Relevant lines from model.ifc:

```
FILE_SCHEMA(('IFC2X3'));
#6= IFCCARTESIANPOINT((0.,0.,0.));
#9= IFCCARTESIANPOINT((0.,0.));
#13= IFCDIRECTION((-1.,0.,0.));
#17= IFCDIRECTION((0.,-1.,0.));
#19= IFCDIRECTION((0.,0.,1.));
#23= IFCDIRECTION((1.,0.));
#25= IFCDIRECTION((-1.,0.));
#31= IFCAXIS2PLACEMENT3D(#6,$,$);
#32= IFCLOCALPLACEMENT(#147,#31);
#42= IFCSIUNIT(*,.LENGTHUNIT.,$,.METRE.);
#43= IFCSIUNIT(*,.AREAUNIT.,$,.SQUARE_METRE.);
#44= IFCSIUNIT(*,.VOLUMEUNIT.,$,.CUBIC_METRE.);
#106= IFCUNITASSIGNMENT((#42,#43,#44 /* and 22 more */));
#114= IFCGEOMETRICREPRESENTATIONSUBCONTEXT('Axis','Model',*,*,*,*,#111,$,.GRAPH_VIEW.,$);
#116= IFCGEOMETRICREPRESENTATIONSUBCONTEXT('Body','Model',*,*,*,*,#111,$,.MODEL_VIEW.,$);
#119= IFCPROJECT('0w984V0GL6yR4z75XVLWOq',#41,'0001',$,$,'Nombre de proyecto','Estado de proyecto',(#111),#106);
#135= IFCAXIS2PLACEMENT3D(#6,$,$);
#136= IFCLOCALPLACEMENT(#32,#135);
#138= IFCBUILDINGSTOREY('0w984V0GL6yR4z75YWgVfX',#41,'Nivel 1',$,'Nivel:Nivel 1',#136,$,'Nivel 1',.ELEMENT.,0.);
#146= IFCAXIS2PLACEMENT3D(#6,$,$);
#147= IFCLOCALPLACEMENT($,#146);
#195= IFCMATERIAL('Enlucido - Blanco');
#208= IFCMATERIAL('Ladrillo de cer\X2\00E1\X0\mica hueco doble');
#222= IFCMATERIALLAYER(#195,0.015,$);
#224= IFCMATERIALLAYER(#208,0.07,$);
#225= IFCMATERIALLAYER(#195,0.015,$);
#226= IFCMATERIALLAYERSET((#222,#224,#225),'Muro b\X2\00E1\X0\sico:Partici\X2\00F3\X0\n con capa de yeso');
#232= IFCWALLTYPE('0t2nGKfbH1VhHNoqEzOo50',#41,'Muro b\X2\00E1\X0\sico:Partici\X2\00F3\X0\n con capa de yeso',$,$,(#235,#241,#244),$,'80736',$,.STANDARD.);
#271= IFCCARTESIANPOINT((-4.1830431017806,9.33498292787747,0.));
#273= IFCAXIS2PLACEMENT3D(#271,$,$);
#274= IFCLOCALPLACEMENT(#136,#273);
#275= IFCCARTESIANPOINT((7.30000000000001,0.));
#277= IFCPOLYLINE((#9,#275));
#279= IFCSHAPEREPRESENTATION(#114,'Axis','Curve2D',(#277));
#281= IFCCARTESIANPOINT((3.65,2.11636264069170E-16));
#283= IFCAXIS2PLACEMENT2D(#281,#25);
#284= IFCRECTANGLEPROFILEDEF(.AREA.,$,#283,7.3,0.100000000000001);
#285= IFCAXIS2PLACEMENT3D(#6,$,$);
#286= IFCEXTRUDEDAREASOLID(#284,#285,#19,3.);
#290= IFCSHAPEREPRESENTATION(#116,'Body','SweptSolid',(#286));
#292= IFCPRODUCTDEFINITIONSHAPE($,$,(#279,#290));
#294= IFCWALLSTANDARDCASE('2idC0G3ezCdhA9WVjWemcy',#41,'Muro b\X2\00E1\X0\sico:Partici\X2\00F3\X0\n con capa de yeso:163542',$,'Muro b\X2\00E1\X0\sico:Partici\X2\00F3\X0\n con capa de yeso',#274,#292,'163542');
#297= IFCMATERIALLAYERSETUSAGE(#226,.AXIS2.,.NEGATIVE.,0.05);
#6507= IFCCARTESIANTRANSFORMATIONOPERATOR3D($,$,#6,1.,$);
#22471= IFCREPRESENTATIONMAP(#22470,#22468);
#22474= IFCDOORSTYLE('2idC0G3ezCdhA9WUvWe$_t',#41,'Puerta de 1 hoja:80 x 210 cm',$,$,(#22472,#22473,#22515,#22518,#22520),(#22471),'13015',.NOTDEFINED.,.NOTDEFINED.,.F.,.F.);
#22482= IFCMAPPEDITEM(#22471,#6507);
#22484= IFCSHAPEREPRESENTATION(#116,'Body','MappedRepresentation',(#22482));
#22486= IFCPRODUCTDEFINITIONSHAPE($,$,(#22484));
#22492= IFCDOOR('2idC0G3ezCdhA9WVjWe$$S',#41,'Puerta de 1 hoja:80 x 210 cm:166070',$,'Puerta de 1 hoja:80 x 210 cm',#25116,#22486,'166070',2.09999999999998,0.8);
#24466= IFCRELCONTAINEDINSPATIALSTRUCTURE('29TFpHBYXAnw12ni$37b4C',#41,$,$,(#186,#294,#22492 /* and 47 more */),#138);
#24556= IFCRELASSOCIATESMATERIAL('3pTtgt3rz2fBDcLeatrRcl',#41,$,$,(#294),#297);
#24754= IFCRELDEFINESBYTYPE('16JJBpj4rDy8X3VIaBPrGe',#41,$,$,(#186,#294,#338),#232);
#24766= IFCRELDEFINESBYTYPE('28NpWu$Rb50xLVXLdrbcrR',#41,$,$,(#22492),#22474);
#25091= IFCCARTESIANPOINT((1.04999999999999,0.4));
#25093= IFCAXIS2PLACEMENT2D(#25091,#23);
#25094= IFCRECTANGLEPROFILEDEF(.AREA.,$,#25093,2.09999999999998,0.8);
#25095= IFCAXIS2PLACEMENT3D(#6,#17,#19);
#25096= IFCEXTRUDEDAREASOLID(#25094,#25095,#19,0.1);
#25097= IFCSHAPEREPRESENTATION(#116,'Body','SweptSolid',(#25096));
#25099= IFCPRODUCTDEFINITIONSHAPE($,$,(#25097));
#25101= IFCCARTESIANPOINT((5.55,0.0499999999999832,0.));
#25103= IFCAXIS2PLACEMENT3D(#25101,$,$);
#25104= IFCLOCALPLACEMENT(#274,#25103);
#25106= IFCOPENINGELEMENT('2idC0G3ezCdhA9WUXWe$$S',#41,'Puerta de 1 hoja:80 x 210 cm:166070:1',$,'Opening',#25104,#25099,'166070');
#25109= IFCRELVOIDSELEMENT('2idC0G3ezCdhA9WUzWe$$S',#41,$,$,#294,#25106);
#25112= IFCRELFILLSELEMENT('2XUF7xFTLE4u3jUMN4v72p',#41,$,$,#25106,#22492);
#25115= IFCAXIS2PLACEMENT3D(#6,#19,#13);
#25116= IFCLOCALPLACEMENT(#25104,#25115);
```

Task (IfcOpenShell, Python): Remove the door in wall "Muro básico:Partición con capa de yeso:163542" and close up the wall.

```python
import ifcopenshell
import ifcopenshell.api.feature
import ifcopenshell.api.root
import ifcopenshell.geom
import ifcopenshell.util.shape

model = ifcopenshell.open("model.ifc")
settings = ifcopenshell.geom.settings()


def volume(element):
    """Net volume in cubic metres, openings subtracted."""
    shape = ifcopenshell.geom.create_shape(settings, element)
    return ifcopenshell.util.shape.get_volume(shape.geometry)


door = model.by_guid("2idC0G3ezCdhA9WVjWe$$S")
opening = door.FillsVoids[0].RelatingOpeningElement
wall = opening.VoidsElements[0].RelatingBuildingElement
before = volume(wall)

ifcopenshell.api.root.remove_product(model, product=door)
ifcopenshell.api.feature.remove_feature(model, feature=opening)

after = volume(wall)

print(f"wall volume {before:.3f} -> {after:.3f} m3")

model.write("model-out.ifc")
```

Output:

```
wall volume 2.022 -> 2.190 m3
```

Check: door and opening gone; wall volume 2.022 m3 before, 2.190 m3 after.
